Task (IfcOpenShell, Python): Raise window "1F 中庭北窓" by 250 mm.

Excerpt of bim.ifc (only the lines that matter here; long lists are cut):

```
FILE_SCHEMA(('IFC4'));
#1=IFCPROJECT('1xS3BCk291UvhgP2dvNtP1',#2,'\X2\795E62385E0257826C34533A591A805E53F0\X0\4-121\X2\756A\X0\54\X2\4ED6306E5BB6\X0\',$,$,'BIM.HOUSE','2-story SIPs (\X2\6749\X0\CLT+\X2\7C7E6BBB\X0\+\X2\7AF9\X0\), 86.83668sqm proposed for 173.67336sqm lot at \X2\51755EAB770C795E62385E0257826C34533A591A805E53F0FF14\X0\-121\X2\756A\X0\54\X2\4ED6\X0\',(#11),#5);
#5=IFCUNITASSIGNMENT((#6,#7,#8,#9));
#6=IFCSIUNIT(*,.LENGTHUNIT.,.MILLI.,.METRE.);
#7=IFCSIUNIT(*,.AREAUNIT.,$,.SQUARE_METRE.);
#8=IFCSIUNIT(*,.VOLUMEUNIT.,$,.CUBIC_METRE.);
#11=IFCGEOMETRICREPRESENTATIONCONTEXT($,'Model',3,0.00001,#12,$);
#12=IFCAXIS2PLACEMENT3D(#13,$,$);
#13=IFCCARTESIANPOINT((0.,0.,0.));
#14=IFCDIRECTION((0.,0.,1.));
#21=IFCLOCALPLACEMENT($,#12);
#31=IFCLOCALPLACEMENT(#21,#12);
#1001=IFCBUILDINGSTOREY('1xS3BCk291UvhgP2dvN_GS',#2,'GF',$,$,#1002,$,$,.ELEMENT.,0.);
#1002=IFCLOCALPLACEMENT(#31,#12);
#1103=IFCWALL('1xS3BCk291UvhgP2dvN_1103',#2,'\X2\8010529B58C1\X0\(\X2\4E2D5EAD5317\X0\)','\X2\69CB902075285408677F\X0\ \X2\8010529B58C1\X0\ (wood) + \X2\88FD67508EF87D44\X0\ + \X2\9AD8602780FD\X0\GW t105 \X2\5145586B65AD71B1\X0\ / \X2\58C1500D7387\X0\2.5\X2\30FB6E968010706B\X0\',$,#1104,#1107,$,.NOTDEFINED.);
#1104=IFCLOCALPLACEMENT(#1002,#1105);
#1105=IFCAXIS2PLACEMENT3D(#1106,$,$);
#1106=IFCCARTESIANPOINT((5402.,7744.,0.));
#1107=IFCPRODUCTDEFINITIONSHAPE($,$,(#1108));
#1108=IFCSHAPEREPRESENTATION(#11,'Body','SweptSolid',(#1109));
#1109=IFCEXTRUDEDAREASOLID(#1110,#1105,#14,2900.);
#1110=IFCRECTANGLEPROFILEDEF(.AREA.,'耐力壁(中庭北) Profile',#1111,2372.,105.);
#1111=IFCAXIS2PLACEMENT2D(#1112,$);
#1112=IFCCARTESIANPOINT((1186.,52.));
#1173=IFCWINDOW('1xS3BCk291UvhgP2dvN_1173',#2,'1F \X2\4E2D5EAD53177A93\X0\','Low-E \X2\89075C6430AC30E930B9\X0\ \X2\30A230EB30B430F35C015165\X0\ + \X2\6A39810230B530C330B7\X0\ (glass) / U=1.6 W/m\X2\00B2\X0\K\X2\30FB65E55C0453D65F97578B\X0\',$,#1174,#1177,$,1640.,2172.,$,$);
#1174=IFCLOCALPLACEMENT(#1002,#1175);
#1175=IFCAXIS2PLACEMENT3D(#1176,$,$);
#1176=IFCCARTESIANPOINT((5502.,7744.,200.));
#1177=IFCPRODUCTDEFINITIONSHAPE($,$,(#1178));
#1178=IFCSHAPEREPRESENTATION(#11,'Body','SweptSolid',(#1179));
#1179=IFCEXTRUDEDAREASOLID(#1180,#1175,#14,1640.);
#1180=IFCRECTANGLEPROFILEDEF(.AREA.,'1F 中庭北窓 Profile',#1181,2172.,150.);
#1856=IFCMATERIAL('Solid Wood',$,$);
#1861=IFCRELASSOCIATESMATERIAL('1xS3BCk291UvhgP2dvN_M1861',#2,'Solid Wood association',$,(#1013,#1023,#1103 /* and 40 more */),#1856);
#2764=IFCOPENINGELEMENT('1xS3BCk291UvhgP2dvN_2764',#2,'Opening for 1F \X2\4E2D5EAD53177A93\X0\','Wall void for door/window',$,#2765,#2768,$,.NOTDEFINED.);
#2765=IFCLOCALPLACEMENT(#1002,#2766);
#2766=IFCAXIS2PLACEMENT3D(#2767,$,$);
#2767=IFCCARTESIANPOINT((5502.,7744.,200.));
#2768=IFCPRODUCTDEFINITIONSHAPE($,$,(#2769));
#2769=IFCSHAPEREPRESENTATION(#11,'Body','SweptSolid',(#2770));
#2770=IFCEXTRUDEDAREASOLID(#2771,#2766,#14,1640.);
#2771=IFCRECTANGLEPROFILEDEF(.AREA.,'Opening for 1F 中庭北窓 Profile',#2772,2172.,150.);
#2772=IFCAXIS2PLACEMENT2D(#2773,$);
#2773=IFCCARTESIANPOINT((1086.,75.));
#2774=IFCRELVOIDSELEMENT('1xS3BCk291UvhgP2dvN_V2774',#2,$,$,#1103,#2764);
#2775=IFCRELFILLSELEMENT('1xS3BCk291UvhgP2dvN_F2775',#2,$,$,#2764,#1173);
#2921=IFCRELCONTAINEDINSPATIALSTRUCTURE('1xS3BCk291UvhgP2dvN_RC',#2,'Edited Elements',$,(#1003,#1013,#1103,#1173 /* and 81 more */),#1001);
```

```python
import numpy as np
import ifcopenshell
import ifcopenshell.api.geometry
import ifcopenshell.util.placement
import ifcopenshell.util.unit

model = ifcopenshell.open("bim.ifc")
unit_scale = ifcopenshell.util.unit.calculate_unit_scale(model)

window = model.by_guid("1xS3BCk291UvhgP2dvN_1173")
opening = window.FillsVoids[0].RelatingOpeningElement
dz = 250.0

shift = np.array([0.0, 0.0, dz])
# The window is not placed relative to its opening, so move both.
for product in (opening, window):
    matrix = ifcopenshell.util.placement.get_local_placement(product.ObjectPlacement)
    matrix[:3, 3] += shift
    ifcopenshell.api.geometry.edit_object_placement(model, product=product, matrix=matrix, is_si=False)

print(f"moved by {dz * unit_scale:+.3f} m")

model.write("bim_updated.ifc")
```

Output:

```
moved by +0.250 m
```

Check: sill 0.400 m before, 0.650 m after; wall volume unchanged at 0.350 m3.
